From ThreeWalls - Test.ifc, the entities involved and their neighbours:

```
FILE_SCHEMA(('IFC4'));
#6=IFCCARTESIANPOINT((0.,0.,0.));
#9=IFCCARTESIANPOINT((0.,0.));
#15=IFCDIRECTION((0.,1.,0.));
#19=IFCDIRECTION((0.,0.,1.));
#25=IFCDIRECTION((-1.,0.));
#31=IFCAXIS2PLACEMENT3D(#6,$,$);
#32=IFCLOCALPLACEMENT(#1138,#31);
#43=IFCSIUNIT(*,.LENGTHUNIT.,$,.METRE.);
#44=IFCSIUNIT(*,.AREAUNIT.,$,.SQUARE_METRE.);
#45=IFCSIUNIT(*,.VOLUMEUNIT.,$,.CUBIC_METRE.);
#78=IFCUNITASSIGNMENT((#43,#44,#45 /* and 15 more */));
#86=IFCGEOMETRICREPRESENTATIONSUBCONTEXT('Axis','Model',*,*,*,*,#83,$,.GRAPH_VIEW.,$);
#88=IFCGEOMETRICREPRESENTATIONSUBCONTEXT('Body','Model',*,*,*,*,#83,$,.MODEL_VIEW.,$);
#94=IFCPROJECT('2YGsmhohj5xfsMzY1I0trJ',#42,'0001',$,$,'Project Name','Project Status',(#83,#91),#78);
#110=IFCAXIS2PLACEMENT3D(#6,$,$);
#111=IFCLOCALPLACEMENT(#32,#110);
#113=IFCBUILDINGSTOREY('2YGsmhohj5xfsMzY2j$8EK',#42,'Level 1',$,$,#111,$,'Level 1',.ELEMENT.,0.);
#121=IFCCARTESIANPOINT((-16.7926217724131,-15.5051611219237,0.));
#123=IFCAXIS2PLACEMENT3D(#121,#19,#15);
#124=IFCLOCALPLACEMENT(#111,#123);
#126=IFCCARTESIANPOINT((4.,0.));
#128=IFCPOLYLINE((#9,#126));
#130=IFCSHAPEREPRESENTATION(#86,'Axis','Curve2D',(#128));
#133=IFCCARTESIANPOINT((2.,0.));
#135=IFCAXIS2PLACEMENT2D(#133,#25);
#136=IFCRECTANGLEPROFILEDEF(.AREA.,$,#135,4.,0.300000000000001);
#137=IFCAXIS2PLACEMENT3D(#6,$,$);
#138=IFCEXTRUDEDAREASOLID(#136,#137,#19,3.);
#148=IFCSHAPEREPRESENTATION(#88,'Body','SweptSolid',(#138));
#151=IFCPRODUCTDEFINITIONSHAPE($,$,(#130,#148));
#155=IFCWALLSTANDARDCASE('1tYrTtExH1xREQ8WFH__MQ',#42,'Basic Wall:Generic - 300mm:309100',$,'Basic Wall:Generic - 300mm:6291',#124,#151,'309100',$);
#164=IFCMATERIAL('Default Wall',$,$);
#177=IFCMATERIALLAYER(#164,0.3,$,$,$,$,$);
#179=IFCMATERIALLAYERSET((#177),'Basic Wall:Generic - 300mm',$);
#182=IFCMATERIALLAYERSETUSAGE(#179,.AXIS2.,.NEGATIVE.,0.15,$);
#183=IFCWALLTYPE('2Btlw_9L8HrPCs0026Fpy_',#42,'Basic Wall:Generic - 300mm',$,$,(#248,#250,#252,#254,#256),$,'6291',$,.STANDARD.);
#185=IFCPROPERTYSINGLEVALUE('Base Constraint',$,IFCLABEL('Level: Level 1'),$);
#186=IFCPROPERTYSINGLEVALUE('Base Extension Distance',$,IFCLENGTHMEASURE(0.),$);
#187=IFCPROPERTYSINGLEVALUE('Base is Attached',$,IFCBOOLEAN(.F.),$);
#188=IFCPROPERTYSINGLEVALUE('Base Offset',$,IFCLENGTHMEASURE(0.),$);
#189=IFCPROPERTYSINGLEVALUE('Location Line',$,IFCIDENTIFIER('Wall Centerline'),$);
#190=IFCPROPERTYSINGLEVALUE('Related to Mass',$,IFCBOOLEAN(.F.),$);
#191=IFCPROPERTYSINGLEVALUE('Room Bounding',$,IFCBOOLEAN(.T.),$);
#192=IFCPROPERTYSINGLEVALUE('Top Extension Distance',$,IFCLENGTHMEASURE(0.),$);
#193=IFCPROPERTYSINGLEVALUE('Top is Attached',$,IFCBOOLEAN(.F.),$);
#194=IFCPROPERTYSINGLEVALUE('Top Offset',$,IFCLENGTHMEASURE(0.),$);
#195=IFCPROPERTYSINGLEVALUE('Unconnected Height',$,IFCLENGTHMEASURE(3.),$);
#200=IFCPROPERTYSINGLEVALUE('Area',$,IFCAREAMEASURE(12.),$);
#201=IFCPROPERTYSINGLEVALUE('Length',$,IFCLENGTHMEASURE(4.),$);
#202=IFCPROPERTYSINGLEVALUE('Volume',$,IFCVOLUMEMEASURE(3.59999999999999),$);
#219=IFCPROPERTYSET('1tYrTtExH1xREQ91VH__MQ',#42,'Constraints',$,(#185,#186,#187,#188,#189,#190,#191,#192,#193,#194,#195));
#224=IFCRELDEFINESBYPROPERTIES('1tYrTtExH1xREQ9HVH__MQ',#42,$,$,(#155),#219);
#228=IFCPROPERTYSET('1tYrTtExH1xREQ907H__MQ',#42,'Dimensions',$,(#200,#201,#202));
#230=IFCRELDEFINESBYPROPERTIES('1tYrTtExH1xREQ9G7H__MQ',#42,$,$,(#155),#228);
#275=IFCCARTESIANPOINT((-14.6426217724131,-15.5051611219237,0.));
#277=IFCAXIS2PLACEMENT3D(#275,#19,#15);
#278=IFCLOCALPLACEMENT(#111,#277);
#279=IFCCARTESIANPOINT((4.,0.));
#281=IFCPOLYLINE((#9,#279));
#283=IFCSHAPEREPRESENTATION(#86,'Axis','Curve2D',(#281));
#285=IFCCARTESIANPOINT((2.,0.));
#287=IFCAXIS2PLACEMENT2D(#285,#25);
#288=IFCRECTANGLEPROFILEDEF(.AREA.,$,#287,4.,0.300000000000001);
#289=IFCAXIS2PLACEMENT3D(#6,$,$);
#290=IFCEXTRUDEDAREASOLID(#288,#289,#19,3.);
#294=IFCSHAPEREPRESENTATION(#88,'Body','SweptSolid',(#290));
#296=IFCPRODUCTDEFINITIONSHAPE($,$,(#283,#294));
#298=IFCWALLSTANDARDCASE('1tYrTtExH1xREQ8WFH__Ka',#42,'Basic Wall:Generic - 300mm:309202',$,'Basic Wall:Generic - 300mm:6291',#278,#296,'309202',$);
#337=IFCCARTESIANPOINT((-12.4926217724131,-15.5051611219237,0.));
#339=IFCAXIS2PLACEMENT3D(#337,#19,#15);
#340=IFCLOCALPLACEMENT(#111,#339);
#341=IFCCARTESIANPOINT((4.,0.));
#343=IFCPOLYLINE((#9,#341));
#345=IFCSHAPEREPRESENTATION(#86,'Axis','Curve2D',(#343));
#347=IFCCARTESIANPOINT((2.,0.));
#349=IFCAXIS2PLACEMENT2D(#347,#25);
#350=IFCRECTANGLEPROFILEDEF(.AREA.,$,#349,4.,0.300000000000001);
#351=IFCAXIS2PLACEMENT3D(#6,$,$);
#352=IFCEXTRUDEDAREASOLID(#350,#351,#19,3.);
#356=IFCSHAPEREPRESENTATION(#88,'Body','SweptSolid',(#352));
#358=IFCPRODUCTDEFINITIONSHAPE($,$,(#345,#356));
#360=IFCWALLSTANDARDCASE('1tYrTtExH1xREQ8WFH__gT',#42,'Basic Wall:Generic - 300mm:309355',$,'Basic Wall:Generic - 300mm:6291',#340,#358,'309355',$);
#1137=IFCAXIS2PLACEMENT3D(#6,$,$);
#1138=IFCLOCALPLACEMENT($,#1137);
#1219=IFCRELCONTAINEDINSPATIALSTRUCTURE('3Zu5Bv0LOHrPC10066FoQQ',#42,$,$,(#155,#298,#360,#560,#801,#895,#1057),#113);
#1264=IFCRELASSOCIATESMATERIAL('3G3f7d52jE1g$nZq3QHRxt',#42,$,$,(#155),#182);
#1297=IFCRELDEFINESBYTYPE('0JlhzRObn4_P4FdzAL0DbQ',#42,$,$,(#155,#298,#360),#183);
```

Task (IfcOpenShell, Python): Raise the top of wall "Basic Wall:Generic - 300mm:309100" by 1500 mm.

```python
import ifcopenshell
import ifcopenshell.api.pset
import ifcopenshell.geom
import ifcopenshell.util.element
import ifcopenshell.util.representation
import ifcopenshell.util.shape
import ifcopenshell.util.unit

model = ifcopenshell.open("ThreeWalls - Test.ifc")
unit_scale = ifcopenshell.util.unit.calculate_unit_scale(model)
area_scale = ifcopenshell.util.unit.calculate_unit_scale(model, "AREAUNIT")
volume_scale = ifcopenshell.util.unit.calculate_unit_scale(model, "VOLUMEUNIT")
settings = ifcopenshell.geom.settings()


def volume(element):
    """Net volume in cubic metres, openings subtracted."""
    shape = ifcopenshell.geom.create_shape(settings, element)
    return ifcopenshell.util.shape.get_volume(shape.geometry)


wall = model.by_id(155)
before = volume(wall)

body = ifcopenshell.util.representation.get_representation(wall, "Model", "Body")
solid = body.Items[0]
old_height = solid.Depth
solid.Depth += 1.5 / unit_scale
after = volume(wall)
thickness = 0.3  # wall thickness in metres

# Update the stored height, areas and volumes.
pset = model.by_id(ifcopenshell.util.element.get_pset(wall, "Constraints", should_inherit=False)["id"])
ifcopenshell.api.pset.edit_pset(model, pset=pset, properties={
    "Unconnected Height": model.create_entity("IfcLengthMeasure", solid.Depth),
})
pset = model.by_id(ifcopenshell.util.element.get_pset(wall, "Dimensions", should_inherit=False)["id"])
ifcopenshell.api.pset.edit_pset(model, pset=pset, properties={
    "Area": model.create_entity("IfcAreaMeasure", after / thickness / area_scale),
    "Volume": model.create_entity("IfcVolumeMeasure", after / volume_scale),
})

print(f"height {old_height:g} -> {solid.Depth:g}, volume {before:.3f} -> {after:.3f} m3")

model.write("ThreeWalls - Test_v2.ifc")
```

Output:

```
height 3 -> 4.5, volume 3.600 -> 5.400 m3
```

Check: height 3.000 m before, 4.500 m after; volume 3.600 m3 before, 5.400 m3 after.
